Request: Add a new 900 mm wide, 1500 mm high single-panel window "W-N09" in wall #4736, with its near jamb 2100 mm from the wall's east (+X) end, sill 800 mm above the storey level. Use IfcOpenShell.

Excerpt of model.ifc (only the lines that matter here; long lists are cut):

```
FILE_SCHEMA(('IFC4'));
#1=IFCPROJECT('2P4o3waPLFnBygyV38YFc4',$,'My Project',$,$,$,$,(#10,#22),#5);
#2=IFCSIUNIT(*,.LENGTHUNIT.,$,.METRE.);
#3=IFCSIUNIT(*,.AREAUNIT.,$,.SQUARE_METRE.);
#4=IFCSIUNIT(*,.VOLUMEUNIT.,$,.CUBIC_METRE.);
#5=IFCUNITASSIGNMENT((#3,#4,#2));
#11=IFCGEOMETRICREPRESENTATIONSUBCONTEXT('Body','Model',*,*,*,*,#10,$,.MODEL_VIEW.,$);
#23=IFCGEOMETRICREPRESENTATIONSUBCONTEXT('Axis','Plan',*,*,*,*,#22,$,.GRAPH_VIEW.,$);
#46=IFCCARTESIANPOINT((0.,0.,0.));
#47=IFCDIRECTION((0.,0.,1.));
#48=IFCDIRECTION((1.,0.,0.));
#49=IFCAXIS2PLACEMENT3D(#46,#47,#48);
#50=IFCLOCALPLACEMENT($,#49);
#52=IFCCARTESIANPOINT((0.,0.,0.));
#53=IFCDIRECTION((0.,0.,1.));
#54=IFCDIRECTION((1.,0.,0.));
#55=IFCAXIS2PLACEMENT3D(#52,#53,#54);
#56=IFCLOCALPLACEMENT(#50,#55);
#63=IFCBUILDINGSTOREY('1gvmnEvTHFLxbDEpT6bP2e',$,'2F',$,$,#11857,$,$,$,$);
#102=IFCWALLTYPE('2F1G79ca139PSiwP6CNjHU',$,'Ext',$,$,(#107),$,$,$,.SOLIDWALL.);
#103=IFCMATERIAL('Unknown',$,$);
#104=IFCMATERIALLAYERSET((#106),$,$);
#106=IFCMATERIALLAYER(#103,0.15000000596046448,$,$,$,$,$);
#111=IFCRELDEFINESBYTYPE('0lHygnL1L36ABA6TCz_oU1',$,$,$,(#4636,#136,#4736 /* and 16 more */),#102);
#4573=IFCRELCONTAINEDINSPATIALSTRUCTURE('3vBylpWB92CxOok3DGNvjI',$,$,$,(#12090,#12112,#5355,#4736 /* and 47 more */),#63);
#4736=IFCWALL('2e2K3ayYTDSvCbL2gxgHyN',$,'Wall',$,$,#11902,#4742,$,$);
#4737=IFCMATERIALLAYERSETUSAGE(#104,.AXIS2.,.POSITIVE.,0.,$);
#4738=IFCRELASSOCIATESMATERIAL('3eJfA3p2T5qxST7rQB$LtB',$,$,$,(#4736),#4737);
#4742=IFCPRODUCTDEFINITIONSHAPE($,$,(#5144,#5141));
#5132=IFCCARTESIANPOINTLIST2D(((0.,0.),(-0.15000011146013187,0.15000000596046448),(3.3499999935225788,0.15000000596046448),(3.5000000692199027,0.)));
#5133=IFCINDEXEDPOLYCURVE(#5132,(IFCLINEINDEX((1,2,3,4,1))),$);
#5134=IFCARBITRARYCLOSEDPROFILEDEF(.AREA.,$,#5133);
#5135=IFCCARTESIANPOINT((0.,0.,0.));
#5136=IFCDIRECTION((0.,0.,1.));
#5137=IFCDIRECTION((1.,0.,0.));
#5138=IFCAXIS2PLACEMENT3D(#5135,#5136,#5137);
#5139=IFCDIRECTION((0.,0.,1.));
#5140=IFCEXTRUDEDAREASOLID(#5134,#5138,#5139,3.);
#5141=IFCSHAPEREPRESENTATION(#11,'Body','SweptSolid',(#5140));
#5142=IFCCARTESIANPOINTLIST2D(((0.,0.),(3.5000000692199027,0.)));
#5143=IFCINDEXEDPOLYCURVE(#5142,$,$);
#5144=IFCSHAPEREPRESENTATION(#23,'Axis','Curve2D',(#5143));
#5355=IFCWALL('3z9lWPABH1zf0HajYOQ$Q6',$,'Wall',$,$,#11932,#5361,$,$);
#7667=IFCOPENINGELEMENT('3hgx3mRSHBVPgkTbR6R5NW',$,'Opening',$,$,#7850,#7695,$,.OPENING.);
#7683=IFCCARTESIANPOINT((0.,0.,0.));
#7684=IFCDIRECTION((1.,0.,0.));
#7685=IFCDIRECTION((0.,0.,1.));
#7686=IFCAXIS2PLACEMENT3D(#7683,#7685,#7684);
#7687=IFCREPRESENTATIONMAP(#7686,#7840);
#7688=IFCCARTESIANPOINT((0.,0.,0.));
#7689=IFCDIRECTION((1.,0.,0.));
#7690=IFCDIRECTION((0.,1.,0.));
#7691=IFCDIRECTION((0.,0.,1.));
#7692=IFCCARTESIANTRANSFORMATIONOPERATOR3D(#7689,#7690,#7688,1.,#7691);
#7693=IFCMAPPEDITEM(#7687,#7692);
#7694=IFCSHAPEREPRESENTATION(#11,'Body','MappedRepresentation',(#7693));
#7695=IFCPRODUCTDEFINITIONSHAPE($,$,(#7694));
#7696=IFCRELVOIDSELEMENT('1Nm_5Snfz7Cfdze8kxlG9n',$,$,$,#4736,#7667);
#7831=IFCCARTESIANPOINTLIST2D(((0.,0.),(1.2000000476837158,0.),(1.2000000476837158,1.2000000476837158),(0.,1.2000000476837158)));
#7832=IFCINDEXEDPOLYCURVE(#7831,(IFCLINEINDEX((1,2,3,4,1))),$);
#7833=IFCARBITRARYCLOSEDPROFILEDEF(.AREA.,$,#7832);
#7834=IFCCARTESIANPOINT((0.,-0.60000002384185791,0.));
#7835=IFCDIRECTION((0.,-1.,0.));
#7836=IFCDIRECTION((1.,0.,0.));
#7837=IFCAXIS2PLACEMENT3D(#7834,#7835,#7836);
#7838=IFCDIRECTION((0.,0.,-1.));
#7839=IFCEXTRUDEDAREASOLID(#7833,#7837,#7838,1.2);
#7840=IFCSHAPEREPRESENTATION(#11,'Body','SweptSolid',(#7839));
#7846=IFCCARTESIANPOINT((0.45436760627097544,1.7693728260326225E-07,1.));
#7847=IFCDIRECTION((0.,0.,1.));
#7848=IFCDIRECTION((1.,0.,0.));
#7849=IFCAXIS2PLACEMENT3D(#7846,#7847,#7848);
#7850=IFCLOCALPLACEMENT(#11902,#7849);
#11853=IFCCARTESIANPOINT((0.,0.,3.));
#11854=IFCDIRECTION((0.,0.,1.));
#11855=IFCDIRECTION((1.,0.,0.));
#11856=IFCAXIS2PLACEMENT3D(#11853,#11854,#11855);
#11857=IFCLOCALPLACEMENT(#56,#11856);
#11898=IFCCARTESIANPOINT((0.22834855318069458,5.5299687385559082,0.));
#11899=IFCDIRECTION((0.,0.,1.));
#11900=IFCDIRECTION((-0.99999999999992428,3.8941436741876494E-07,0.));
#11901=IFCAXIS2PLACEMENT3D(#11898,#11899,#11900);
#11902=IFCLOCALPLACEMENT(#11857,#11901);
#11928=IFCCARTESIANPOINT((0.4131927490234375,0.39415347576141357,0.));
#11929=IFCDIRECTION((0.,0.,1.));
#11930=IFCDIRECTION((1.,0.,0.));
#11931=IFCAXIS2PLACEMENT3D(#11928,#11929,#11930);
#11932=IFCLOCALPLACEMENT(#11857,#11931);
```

```python
import numpy as np
import ifcopenshell
import ifcopenshell.api.feature
import ifcopenshell.api.geometry
import ifcopenshell.api.root
import ifcopenshell.api.spatial
import ifcopenshell.geom
import ifcopenshell.util.element
import ifcopenshell.util.placement
import ifcopenshell.util.representation
import ifcopenshell.util.shape
import ifcopenshell.util.unit

model = ifcopenshell.open("model.ifc")
unit_scale = ifcopenshell.util.unit.calculate_unit_scale(model)
settings = ifcopenshell.geom.settings()


def volume(element):
    """Net volume in cubic metres, openings subtracted."""
    shape = ifcopenshell.geom.create_shape(settings, element)
    return ifcopenshell.util.shape.get_volume(shape.geometry)


wall = model.by_guid("2e2K3ayYTDSvCbL2gxgHyN")
storey = ifcopenshell.util.element.get_container(wall, ifc_class="IfcBuildingStorey")
context = ifcopenshell.util.representation.get_context(model, "Model", "Body", "MODEL_VIEW")
before = volume(wall)

width, height, from_end, sill = 0.9, 1.5, 2.1, 0.8  # metres

# The wall runs along its own X axis, and the end named is its -X end.
wall_shape = ifcopenshell.geom.create_shape(settings, wall)
x, y, z = ifcopenshell.util.shape.get_vertices(wall_shape.geometry).T
start = x.min() + from_end
face, thickness = float(y.min()), float(y.max() - y.min())
wall_matrix = ifcopenshell.util.placement.get_local_placement(wall.ObjectPlacement)
level = ifcopenshell.util.placement.get_local_placement(storey.ObjectPlacement)[2, 3]


def in_wall(x, y):
    """Placement at x, y metres in the wall's axes, at sill height."""
    matrix = wall_matrix.copy()
    matrix[:, 3] = wall_matrix @ np.array([x / unit_scale, y / unit_scale, 0.0, 1.0])
    matrix[2, 3] = level + sill / unit_scale
    return matrix


# Opening: a box that overshoots both wall faces by 50 mm.
opening = ifcopenshell.api.root.create_entity(model, ifc_class="IfcOpeningElement", predefined_type="OPENING")
box = ifcopenshell.api.geometry.add_wall_representation(
    model, context=context, length=width, height=height, thickness=thickness + 0.1
)
ifcopenshell.api.geometry.assign_representation(model, product=opening, representation=box)
ifcopenshell.api.geometry.edit_object_placement(model, product=opening, matrix=in_wall(start, face - 0.05), is_si=False)
ifcopenshell.api.feature.add_feature(model, feature=opening, element=wall)

window = ifcopenshell.api.root.create_entity(model, ifc_class="IfcWindow", name="W-N09", predefined_type="WINDOW")
window.OverallWidth, window.OverallHeight = width / unit_scale, height / unit_scale
window.PartitioningType = "SINGLE_PANEL"
body = ifcopenshell.api.geometry.add_window_representation(
    model,
    context=context,
    overall_width=window.OverallWidth,
    overall_height=window.OverallHeight,
    partition_type="SINGLE_PANEL",
)
ifcopenshell.api.geometry.assign_representation(model, product=window, representation=body)
ifcopenshell.api.spatial.assign_container(model, products=[window], relating_structure=storey)
ifcopenshell.api.feature.add_filling(model, opening=opening, element=window)

# Centre the window in the wall's thickness.
ifcopenshell.api.geometry.edit_object_placement(model, product=window, matrix=in_wall(start, face), is_si=False)
window_shape = ifcopenshell.geom.create_shape(settings, window)
depth = ifcopenshell.util.shape.get_vertices(window_shape.geometry)[:, 1]
offset = face + thickness / 2 - (depth.min() + depth.max()) / 2
ifcopenshell.api.geometry.edit_object_placement(model, product=window, matrix=in_wall(start, offset), is_si=False)

after = volume(wall)

print(f"wall volume {before:.3f} -> {after:.3f} m3")

model.write("model_rev.ifc")
```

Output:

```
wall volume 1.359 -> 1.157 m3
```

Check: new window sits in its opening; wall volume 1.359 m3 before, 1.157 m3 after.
